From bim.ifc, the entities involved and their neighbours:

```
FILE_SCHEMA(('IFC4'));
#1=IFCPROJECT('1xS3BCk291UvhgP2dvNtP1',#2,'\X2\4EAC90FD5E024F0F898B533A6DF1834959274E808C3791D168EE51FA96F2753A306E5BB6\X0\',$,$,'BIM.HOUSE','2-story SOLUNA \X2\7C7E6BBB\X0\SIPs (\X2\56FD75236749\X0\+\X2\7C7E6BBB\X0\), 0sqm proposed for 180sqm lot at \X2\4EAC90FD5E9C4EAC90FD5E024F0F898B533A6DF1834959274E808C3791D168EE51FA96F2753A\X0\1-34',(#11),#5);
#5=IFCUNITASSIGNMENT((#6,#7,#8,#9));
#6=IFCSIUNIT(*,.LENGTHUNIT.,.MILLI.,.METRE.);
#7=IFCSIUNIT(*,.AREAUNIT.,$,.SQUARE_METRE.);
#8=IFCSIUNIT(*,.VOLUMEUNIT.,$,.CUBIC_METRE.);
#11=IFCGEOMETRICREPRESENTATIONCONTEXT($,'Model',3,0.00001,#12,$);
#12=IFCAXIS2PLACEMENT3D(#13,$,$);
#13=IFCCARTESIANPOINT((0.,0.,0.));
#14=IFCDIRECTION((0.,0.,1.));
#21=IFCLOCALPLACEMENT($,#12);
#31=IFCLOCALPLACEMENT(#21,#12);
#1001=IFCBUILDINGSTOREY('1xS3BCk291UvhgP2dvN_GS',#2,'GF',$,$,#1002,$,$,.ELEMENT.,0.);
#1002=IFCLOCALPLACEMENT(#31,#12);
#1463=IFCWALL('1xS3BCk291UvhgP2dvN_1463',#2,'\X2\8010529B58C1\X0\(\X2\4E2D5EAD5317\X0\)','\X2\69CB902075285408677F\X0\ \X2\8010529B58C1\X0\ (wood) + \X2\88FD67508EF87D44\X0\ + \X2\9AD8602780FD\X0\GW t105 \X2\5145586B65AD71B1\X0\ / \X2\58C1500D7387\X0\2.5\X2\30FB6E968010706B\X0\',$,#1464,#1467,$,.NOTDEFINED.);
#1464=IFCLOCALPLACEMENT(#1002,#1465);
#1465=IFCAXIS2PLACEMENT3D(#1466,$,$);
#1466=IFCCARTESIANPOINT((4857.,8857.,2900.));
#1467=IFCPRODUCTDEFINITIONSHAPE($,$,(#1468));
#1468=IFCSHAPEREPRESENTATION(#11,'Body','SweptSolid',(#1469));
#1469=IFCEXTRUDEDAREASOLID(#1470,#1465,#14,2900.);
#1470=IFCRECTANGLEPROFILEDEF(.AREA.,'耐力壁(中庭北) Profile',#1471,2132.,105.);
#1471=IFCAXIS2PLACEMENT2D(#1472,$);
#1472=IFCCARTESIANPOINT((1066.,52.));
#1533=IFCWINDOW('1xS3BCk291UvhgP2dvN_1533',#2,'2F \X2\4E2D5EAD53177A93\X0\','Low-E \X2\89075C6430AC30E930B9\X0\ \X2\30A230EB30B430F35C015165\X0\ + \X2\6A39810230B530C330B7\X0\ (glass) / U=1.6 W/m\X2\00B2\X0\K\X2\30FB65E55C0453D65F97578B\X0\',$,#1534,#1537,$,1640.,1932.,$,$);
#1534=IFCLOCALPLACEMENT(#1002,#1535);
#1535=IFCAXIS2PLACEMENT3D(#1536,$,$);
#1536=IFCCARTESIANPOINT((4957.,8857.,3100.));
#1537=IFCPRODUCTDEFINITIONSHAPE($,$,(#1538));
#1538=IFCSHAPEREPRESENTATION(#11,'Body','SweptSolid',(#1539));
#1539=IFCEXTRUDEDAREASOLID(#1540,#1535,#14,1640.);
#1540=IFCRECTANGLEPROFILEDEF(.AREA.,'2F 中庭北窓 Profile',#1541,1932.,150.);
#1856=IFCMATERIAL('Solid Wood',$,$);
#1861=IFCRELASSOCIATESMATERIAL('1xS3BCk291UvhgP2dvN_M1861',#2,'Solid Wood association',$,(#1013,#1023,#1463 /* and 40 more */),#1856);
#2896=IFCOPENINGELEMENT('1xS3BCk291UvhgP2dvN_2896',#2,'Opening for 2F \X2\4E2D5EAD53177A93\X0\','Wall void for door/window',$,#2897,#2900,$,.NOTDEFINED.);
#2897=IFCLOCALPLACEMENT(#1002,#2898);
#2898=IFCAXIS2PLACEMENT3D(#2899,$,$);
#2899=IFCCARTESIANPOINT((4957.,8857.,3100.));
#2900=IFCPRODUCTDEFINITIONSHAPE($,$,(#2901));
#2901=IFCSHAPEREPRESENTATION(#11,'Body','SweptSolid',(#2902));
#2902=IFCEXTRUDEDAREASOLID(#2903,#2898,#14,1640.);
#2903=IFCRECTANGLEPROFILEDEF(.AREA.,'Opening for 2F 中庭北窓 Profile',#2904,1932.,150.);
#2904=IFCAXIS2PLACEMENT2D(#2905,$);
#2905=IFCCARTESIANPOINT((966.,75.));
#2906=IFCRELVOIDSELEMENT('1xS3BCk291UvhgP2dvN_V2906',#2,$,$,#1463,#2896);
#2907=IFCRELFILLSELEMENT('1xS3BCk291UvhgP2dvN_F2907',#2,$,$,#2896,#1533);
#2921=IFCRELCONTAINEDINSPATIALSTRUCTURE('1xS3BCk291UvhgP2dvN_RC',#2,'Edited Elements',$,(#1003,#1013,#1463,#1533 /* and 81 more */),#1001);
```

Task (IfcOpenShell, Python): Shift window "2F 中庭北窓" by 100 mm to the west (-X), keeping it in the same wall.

```python
import ifcopenshell
import ifcopenshell.api.geometry
import ifcopenshell.util.placement
import ifcopenshell.util.unit

model = ifcopenshell.open("bim.ifc")
unit_scale = ifcopenshell.util.unit.calculate_unit_scale(model)

window = model.by_guid("1xS3BCk291UvhgP2dvN_1533")
opening = window.FillsVoids[0].RelatingOpeningElement
wall = opening.VoidsElements[0].RelatingBuildingElement

wall_matrix = ifcopenshell.util.placement.get_local_placement(wall.ObjectPlacement)
shift = wall_matrix[:3, 0] * -0.1 / unit_scale
before = ifcopenshell.util.placement.get_local_placement(window.ObjectPlacement)[:3, 3].copy()

# The window is not placed relative to its opening, so move both.
for product in (opening, window):
    matrix = ifcopenshell.util.placement.get_local_placement(product.ObjectPlacement)
    matrix[:3, 3] += shift
    ifcopenshell.api.geometry.edit_object_placement(model, product=product, matrix=matrix, is_si=False)

after = ifcopenshell.util.placement.get_local_placement(window.ObjectPlacement)[:3, 3]
print("window moved by", (after - before).round(3) + 0.0)

model.write("bim_updated.ifc")
```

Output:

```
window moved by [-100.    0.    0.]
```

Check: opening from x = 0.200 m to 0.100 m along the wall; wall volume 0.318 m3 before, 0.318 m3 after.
